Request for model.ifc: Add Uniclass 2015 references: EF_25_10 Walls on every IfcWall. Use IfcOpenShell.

First a look at what the model holds.

```python
import ifcopenshell

model = ifcopenshell.open("model.ifc")
print(model.schema)
print("classifications:", [c.Name for c in model.by_type("IfcClassification")])
for ifc_class in ("IfcDoor", "IfcRoof", "IfcStair", "IfcWall", "IfcWindow"):
    print(ifc_class, len(model.by_type(ifc_class)))
```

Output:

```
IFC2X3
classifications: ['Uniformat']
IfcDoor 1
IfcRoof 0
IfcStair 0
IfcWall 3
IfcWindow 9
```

```python
import ifcopenshell
import ifcopenshell.api.classification

model = ifcopenshell.open("model.ifc")

# IFC2X3 requires Source and Edition and has no link from the project to the system.
system = model.create_entity("IfcClassification", Source="NBS", Edition="2015", Name="Uniclass 2015")

codes = {
    "IfcWall": ("EF_25_10", "Walls"),
}
for ifc_class, (code, name) in codes.items():
    products = model.by_type(ifc_class)
    ifcopenshell.api.classification.add_reference(
        model, products=products, classification=system, identification=code, name=name
    )
    print(code, len(products))

model.write("model-out.ifc")
```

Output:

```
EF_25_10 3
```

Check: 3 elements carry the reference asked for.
